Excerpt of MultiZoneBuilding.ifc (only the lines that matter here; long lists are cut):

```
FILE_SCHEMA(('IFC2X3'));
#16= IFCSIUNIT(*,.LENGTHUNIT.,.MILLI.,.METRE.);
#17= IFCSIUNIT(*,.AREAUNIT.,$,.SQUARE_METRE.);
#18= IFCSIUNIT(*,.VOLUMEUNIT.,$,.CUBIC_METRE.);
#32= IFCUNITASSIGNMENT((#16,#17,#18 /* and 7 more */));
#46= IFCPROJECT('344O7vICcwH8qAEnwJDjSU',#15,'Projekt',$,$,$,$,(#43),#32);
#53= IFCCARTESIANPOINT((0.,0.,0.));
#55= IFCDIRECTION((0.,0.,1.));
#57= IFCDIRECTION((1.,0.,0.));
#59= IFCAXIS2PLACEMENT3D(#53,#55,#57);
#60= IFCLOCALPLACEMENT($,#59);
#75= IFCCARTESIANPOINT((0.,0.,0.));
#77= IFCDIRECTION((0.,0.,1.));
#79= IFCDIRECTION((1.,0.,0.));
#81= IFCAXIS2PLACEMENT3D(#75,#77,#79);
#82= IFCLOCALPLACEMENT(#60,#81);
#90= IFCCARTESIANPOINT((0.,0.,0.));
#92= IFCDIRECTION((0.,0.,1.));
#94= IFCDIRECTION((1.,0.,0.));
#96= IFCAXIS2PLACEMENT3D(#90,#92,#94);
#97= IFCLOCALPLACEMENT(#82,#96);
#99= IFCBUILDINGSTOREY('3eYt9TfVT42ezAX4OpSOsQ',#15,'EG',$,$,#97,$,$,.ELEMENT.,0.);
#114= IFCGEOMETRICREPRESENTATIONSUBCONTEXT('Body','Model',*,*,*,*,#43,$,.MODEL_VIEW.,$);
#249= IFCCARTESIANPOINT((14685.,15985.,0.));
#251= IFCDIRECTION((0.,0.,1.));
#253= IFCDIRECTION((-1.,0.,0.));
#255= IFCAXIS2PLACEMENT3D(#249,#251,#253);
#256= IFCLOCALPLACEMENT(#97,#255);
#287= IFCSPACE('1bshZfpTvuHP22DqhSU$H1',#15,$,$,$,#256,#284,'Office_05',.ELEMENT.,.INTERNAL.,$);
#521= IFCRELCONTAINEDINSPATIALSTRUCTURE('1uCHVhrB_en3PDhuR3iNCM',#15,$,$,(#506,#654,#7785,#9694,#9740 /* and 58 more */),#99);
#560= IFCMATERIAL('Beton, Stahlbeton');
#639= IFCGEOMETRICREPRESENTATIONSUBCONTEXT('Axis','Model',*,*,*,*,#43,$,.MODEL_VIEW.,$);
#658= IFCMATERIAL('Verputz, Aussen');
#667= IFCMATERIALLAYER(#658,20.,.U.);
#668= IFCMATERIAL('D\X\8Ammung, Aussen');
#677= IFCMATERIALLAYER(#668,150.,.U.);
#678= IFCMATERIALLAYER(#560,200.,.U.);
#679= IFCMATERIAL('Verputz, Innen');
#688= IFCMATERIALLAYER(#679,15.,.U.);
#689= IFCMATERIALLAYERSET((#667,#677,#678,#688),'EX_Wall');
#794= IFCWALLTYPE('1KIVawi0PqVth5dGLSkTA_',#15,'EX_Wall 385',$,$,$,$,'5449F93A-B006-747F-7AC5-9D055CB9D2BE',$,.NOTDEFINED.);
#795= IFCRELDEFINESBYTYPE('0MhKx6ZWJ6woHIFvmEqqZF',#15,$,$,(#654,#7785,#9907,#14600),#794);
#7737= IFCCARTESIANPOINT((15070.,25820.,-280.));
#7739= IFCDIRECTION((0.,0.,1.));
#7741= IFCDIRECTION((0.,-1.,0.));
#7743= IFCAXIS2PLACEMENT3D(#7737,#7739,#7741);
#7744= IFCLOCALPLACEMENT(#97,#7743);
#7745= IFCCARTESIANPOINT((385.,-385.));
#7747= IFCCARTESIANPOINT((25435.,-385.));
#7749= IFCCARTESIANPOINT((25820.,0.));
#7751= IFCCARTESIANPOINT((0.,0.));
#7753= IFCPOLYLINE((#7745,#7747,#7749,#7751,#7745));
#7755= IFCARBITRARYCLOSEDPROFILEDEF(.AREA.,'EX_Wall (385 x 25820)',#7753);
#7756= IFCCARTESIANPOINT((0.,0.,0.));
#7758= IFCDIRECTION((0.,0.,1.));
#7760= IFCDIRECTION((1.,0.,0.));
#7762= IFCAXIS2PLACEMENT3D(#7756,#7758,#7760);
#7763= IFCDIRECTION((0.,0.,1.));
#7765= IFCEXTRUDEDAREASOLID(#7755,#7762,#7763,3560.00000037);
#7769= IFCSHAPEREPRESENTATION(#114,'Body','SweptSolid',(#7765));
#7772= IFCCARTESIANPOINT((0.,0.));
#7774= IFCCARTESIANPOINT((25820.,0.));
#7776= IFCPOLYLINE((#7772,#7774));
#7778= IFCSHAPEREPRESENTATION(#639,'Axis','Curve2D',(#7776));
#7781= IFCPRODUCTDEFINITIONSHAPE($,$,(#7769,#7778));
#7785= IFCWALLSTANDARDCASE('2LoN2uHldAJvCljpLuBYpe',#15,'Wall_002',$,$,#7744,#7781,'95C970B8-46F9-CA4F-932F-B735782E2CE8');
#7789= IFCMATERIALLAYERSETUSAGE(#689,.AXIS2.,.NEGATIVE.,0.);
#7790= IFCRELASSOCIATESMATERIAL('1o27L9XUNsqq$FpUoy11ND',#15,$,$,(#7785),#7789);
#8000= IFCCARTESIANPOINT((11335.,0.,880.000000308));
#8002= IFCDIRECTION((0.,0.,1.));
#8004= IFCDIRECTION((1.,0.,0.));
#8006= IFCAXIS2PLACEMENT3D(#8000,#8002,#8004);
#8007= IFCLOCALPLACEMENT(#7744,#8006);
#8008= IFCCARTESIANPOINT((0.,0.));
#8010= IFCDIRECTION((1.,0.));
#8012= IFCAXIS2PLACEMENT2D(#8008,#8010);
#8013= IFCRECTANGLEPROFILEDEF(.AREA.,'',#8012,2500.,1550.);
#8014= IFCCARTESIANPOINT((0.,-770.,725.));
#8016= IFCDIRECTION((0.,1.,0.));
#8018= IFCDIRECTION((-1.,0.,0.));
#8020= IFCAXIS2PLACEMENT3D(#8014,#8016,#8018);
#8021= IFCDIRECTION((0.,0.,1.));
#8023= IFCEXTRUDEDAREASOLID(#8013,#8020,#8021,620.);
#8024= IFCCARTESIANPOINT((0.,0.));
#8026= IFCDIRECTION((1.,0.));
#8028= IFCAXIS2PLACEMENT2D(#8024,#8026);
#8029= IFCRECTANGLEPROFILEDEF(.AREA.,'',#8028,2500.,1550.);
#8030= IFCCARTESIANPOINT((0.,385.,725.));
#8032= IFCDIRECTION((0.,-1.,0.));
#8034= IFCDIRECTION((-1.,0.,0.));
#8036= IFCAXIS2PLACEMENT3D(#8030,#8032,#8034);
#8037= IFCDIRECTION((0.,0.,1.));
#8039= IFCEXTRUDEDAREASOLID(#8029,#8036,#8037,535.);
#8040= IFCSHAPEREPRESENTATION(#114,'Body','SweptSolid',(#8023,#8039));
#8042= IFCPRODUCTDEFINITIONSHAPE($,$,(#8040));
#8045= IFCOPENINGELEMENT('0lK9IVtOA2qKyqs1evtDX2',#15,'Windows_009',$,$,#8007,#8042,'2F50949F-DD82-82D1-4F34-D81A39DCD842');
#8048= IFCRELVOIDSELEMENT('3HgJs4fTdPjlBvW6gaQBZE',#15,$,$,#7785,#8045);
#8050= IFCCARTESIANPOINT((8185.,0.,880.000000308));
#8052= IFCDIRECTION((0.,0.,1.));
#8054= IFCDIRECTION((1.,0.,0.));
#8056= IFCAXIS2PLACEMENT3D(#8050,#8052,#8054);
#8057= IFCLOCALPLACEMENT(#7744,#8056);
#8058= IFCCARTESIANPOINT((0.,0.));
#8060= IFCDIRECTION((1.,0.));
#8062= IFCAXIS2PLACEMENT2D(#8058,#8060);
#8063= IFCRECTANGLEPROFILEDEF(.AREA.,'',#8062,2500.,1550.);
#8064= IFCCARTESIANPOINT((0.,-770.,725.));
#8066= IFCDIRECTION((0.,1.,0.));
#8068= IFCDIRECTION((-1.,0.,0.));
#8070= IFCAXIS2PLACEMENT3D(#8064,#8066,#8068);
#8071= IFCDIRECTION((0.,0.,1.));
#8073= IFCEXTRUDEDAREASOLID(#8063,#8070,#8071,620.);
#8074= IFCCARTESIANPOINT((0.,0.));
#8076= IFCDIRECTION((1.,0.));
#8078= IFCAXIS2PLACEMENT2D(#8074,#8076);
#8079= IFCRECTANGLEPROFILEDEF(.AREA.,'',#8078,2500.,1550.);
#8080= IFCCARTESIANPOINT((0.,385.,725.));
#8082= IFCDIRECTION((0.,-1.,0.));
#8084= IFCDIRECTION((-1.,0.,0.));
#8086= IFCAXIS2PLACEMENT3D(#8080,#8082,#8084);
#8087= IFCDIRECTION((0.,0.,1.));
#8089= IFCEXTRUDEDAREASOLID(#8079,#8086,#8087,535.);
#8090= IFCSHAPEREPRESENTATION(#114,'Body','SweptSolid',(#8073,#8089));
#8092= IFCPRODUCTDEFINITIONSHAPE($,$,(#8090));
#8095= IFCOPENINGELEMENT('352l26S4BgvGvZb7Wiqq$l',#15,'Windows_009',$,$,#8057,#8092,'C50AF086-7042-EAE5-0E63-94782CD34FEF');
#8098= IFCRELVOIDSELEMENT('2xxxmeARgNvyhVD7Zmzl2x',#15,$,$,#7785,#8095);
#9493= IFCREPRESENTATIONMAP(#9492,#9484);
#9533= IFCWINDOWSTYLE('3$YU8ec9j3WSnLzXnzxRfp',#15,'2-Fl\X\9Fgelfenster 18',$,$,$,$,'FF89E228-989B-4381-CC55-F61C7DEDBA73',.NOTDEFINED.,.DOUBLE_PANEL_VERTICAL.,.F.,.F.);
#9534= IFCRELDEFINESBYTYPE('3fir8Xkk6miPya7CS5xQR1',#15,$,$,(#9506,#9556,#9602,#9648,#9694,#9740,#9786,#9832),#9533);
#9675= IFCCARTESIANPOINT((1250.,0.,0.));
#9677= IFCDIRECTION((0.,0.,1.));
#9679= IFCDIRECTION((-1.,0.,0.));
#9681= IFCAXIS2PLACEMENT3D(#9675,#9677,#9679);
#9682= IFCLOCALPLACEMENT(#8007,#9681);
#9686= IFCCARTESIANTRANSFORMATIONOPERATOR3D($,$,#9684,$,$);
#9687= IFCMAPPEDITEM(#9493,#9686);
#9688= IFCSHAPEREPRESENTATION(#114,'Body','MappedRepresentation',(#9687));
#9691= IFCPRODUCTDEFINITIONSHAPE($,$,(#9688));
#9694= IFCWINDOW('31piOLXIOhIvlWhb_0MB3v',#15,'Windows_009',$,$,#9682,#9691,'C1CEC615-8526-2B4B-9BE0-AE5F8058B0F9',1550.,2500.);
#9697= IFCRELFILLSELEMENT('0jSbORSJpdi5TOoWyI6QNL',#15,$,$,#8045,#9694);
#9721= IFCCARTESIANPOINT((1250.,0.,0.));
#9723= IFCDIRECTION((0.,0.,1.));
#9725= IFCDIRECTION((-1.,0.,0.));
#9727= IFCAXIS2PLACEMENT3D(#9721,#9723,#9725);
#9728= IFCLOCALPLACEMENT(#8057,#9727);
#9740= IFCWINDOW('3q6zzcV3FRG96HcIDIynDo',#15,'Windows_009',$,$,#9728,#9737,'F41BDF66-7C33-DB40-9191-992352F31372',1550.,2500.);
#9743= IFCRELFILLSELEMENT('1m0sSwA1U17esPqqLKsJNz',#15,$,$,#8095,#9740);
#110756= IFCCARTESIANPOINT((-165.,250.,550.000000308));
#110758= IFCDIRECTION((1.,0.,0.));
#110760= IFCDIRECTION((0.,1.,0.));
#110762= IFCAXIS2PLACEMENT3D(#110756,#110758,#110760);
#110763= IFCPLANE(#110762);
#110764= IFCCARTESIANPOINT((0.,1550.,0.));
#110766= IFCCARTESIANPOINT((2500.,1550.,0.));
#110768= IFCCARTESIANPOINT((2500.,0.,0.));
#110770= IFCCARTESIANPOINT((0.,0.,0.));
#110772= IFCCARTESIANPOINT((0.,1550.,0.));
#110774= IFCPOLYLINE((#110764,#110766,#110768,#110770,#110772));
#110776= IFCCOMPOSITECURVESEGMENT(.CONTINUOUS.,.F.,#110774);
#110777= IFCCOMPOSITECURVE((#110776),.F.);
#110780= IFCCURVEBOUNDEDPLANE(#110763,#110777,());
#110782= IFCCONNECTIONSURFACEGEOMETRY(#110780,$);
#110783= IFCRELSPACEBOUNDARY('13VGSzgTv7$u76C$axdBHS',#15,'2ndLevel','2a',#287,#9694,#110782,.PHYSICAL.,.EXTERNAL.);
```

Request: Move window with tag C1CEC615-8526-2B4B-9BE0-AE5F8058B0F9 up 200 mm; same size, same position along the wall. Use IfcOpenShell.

```python
import numpy as np
import ifcopenshell
import ifcopenshell.api.geometry
import ifcopenshell.util.placement
import ifcopenshell.util.unit

model = ifcopenshell.open("MultiZoneBuilding.ifc")
unit_scale = ifcopenshell.util.unit.calculate_unit_scale(model)

window = model.by_id(9694)
opening = window.FillsVoids[0].RelatingOpeningElement
dz = 0.2 / unit_scale

shift = np.array([0.0, 0.0, dz])
# The window is placed relative to its opening, so it follows when the opening moves.
matrix = ifcopenshell.util.placement.get_local_placement(opening.ObjectPlacement)
matrix[:3, 3] += shift
ifcopenshell.api.geometry.edit_object_placement(
    model, product=opening, matrix=matrix, is_si=False, should_transform_children=True
)

# Space boundary surfaces are stored in each space's coordinates; move them too.
for rel in window.ProvidesBoundaries:
    if not rel.ConnectionGeometry:
        continue
    surface = rel.ConnectionGeometry.SurfaceOnRelatingElement.BasisSurface
    space_matrix = ifcopenshell.util.placement.get_local_placement(rel.RelatingSpace.ObjectPlacement)
    point = np.array(surface.Position.Location.Coordinates) + space_matrix[:3, :3].T @ shift
    surface.Position = model.createIfcAxis2Placement3D(
        model.createIfcCartesianPoint(point.tolist()), surface.Position.Axis, surface.Position.RefDirection
    )

print(f"moved by {dz * unit_scale:+.3f} m")

model.write("MultiZoneBuilding_v2.ifc")
```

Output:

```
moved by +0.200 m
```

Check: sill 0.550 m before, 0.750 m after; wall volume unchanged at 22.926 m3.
